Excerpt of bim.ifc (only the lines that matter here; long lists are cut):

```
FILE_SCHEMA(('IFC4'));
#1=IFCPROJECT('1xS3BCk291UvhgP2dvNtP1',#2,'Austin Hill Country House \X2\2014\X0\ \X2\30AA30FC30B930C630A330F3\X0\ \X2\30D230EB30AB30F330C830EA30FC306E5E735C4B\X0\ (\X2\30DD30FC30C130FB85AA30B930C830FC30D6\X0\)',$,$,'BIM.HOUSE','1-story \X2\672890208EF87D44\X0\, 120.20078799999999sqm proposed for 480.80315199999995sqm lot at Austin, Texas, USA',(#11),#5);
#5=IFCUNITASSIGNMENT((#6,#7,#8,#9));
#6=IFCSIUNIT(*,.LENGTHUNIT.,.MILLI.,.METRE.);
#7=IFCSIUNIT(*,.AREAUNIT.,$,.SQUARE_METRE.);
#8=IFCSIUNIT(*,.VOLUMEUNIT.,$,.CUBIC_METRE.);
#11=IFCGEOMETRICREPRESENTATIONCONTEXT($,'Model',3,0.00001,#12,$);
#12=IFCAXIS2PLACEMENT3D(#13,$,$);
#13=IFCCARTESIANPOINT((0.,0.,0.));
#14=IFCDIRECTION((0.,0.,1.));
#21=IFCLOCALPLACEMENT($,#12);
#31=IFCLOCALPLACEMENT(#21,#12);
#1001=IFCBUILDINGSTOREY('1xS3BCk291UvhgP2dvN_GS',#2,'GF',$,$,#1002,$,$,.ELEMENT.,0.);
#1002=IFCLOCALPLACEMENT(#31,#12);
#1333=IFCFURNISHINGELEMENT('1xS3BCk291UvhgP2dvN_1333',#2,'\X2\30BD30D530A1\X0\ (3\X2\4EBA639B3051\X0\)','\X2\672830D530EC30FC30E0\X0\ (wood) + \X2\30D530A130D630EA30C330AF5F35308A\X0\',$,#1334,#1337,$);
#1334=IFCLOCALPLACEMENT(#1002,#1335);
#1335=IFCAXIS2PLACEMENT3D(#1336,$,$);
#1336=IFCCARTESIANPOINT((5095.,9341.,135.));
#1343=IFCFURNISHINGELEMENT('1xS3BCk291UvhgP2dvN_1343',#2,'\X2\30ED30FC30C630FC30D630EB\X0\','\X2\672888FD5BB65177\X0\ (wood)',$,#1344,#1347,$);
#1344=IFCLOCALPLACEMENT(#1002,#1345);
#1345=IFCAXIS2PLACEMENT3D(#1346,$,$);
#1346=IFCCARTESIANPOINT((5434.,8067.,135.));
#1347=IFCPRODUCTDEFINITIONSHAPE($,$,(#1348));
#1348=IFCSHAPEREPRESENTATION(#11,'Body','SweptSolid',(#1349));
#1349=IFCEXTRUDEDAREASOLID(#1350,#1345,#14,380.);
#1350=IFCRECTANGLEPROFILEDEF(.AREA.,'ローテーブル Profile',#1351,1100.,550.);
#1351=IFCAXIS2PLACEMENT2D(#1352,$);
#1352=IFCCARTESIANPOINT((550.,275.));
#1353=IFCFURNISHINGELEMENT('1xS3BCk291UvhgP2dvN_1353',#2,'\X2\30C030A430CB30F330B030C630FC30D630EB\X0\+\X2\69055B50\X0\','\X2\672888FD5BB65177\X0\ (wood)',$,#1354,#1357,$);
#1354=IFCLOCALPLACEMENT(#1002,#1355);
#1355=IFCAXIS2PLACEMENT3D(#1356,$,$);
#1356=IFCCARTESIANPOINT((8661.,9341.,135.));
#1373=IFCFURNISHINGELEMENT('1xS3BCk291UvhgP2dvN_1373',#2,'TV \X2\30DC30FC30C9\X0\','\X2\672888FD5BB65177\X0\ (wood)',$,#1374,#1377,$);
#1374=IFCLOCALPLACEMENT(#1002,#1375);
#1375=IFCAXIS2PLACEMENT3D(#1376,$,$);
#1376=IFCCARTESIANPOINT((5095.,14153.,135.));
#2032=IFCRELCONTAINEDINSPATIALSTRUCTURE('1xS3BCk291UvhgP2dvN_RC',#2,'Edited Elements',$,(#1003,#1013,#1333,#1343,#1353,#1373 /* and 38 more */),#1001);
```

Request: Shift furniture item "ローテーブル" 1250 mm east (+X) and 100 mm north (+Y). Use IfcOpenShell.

```python
import ifcopenshell
import ifcopenshell.api.geometry
import ifcopenshell.util.placement
import ifcopenshell.util.unit

model = ifcopenshell.open("bim.ifc")
unit_scale = ifcopenshell.util.unit.calculate_unit_scale(model)

item = model.by_guid("1xS3BCk291UvhgP2dvN_1343")
matrix = ifcopenshell.util.placement.get_local_placement(item.ObjectPlacement)
matrix[0, 3] += 1.25 / unit_scale
matrix[1, 3] += 0.1 / unit_scale
ifcopenshell.api.geometry.edit_object_placement(model, product=item, matrix=matrix, is_si=False)

print(ifcopenshell.util.placement.get_local_placement(item.ObjectPlacement).round(3) + 0.0)

model.write("bim_updated.ifc")
```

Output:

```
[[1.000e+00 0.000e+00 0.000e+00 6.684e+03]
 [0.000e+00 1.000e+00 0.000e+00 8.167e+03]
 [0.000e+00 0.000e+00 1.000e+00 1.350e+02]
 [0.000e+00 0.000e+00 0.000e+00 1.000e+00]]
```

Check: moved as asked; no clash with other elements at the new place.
